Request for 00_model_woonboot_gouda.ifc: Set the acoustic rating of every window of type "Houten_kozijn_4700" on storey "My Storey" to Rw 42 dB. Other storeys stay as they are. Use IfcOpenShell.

First a look at what the model holds.

```python
import ifcopenshell
import ifcopenshell.util.element

model = ifcopenshell.open("00_model_woonboot_gouda.ifc")
print(model.schema)
storey = next(s for s in model.by_type("IfcBuildingStorey") if s.Name == "My Storey")
windows = [e for e in ifcopenshell.util.element.get_decomposition(storey) if e.is_a("IfcWindow")]
seen = {}
for e in windows:
    element_type = ifcopenshell.util.element.get_type(e)
    key = (element_type.Name if element_type != e and element_type else None, ifcopenshell.util.element.get_pset(e, "Pset_WindowCommon", "AcousticRating"))
    seen[key] = seen.get(key, 0) + 1
for (name, value), count in sorted(seen.items(), key=str):
    print(count, "x", name, "|", value)
```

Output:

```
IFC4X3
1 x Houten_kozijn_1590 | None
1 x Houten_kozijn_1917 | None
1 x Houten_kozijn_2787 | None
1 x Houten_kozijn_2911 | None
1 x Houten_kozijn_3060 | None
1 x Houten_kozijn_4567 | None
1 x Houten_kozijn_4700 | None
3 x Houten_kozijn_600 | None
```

```python
import ifcopenshell
import ifcopenshell.api.pset
import ifcopenshell.util.element

model = ifcopenshell.open("00_model_woonboot_gouda.ifc")

storey = next(s for s in model.by_type("IfcBuildingStorey") if s.Name == "My Storey")
windows = [e for e in ifcopenshell.util.element.get_decomposition(storey) if e.is_a("IfcWindow")]

count = 0
for e in windows:
    element_type = ifcopenshell.util.element.get_type(e)
    if element_type in (None, e) or element_type.Name != "Houten_kozijn_4700":
        continue
    # add_pset returns the element's existing set when there is one.
    pset = ifcopenshell.api.pset.add_pset(model, product=e, name="Pset_WindowCommon")
    ifcopenshell.api.pset.edit_pset(model, pset=pset, properties={"AcousticRating": "Rw 42 dB"})
    count += 1

print(count, "windows updated")

model.write("00_model_woonboot_gouda-out.ifc")
```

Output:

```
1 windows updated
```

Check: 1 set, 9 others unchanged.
